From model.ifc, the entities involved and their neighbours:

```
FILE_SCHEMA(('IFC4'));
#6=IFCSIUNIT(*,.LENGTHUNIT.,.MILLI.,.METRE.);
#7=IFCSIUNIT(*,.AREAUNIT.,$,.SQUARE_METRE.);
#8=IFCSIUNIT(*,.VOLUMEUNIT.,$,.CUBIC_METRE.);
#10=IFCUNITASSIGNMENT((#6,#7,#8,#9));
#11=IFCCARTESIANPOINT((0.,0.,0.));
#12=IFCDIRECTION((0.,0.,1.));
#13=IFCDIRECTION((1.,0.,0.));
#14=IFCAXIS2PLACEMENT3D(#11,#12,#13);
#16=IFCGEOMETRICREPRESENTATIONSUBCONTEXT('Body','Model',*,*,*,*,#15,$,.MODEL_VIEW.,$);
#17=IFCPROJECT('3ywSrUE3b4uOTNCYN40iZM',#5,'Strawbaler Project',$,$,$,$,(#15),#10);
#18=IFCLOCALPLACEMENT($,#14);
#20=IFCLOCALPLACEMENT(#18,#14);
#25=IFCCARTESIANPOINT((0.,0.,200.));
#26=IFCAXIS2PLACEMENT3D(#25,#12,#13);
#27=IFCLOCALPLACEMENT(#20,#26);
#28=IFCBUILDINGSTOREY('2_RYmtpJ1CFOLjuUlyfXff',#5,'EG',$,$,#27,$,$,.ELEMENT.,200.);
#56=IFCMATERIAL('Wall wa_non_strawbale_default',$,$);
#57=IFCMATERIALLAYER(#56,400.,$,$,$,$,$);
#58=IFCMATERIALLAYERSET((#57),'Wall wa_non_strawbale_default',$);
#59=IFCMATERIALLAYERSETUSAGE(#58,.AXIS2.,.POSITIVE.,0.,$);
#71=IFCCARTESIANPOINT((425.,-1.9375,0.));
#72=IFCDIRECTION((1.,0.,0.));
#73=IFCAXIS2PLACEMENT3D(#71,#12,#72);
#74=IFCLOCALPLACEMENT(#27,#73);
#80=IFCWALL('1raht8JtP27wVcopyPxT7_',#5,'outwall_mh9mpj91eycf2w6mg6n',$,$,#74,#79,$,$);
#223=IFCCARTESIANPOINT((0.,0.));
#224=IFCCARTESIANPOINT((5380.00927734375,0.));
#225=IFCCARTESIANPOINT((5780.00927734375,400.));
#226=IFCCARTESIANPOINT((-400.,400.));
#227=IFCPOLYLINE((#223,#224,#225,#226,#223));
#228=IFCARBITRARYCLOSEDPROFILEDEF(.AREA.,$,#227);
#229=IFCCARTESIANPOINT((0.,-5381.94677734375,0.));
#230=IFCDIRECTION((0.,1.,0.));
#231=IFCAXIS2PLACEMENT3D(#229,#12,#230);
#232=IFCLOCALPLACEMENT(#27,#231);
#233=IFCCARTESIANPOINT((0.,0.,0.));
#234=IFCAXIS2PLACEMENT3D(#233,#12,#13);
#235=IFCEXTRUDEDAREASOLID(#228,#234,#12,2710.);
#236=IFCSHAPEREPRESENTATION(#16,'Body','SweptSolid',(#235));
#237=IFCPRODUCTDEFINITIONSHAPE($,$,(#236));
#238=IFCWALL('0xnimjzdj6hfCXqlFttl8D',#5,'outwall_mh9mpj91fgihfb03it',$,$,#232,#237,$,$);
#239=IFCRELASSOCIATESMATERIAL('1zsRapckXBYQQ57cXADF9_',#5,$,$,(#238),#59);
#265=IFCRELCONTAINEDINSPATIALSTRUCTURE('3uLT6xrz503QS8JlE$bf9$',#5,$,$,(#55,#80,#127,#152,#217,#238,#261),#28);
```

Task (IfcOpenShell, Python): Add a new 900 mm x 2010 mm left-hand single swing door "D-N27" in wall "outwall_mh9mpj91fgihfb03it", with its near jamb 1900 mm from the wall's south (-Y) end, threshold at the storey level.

```python
import numpy as np
import ifcopenshell
import ifcopenshell.api.feature
import ifcopenshell.api.geometry
import ifcopenshell.api.root
import ifcopenshell.api.spatial
import ifcopenshell.geom
import ifcopenshell.util.element
import ifcopenshell.util.placement
import ifcopenshell.util.representation
import ifcopenshell.util.shape
import ifcopenshell.util.unit

model = ifcopenshell.open("model.ifc")
unit_scale = ifcopenshell.util.unit.calculate_unit_scale(model)
settings = ifcopenshell.geom.settings()


def volume(element):
    """Net volume in cubic metres, openings subtracted."""
    shape = ifcopenshell.geom.create_shape(settings, element)
    return ifcopenshell.util.shape.get_volume(shape.geometry)


wall = model.by_id(238)
storey = ifcopenshell.util.element.get_container(wall, ifc_class="IfcBuildingStorey")
context = ifcopenshell.util.representation.get_context(model, "Model", "Body", "MODEL_VIEW")
before = volume(wall)

width, height, from_end, sill = 0.9, 2.01, 1.9, 0.0  # metres

# The wall runs along its own X axis, and the end named is its -X end.
wall_shape = ifcopenshell.geom.create_shape(settings, wall)
x, y, z = ifcopenshell.util.shape.get_vertices(wall_shape.geometry).T
start = x.min() + from_end
face, thickness = float(y.min()), float(y.max() - y.min())
wall_matrix = ifcopenshell.util.placement.get_local_placement(wall.ObjectPlacement)
level = ifcopenshell.util.placement.get_local_placement(storey.ObjectPlacement)[2, 3]


def in_wall(x, y):
    """Placement at x, y metres in the wall's axes, at sill height."""
    matrix = wall_matrix.copy()
    matrix[:, 3] = wall_matrix @ np.array([x / unit_scale, y / unit_scale, 0.0, 1.0])
    matrix[2, 3] = level + sill / unit_scale
    return matrix


# Opening: a box that overshoots both wall faces by 50 mm.
opening = ifcopenshell.api.root.create_entity(model, ifc_class="IfcOpeningElement", predefined_type="OPENING")
box = ifcopenshell.api.geometry.add_wall_representation(
    model, context=context, length=width, height=height, thickness=thickness + 0.1
)
ifcopenshell.api.geometry.assign_representation(model, product=opening, representation=box)
ifcopenshell.api.geometry.edit_object_placement(model, product=opening, matrix=in_wall(start, face - 0.05), is_si=False)
ifcopenshell.api.feature.add_feature(model, feature=opening, element=wall)

door = ifcopenshell.api.root.create_entity(model, ifc_class="IfcDoor", name="D-N27", predefined_type="DOOR")
door.OverallWidth, door.OverallHeight = width / unit_scale, height / unit_scale
door.OperationType = "SINGLE_SWING_LEFT"
body = ifcopenshell.api.geometry.add_door_representation(
    model,
    context=context,
    overall_width=door.OverallWidth,
    overall_height=door.OverallHeight,
    operation_type="SINGLE_SWING_LEFT",
    lining_properties={"LiningDepth": thickness / unit_scale, "ThresholdDepth": thickness / unit_scale},
)
ifcopenshell.api.geometry.assign_representation(model, product=door, representation=body)
ifcopenshell.api.spatial.assign_container(model, products=[door], relating_structure=storey)
ifcopenshell.api.feature.add_filling(model, opening=opening, element=door)

# The lining spans the wall, so the door starts at the wall face.
ifcopenshell.api.geometry.edit_object_placement(model, product=door, matrix=in_wall(start, face), is_si=False)

after = volume(wall)

print(f"wall volume {before:.3f} -> {after:.3f} m3")

model.write("model_updated.ifc")
```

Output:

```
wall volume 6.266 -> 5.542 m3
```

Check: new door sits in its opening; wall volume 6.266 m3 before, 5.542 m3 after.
